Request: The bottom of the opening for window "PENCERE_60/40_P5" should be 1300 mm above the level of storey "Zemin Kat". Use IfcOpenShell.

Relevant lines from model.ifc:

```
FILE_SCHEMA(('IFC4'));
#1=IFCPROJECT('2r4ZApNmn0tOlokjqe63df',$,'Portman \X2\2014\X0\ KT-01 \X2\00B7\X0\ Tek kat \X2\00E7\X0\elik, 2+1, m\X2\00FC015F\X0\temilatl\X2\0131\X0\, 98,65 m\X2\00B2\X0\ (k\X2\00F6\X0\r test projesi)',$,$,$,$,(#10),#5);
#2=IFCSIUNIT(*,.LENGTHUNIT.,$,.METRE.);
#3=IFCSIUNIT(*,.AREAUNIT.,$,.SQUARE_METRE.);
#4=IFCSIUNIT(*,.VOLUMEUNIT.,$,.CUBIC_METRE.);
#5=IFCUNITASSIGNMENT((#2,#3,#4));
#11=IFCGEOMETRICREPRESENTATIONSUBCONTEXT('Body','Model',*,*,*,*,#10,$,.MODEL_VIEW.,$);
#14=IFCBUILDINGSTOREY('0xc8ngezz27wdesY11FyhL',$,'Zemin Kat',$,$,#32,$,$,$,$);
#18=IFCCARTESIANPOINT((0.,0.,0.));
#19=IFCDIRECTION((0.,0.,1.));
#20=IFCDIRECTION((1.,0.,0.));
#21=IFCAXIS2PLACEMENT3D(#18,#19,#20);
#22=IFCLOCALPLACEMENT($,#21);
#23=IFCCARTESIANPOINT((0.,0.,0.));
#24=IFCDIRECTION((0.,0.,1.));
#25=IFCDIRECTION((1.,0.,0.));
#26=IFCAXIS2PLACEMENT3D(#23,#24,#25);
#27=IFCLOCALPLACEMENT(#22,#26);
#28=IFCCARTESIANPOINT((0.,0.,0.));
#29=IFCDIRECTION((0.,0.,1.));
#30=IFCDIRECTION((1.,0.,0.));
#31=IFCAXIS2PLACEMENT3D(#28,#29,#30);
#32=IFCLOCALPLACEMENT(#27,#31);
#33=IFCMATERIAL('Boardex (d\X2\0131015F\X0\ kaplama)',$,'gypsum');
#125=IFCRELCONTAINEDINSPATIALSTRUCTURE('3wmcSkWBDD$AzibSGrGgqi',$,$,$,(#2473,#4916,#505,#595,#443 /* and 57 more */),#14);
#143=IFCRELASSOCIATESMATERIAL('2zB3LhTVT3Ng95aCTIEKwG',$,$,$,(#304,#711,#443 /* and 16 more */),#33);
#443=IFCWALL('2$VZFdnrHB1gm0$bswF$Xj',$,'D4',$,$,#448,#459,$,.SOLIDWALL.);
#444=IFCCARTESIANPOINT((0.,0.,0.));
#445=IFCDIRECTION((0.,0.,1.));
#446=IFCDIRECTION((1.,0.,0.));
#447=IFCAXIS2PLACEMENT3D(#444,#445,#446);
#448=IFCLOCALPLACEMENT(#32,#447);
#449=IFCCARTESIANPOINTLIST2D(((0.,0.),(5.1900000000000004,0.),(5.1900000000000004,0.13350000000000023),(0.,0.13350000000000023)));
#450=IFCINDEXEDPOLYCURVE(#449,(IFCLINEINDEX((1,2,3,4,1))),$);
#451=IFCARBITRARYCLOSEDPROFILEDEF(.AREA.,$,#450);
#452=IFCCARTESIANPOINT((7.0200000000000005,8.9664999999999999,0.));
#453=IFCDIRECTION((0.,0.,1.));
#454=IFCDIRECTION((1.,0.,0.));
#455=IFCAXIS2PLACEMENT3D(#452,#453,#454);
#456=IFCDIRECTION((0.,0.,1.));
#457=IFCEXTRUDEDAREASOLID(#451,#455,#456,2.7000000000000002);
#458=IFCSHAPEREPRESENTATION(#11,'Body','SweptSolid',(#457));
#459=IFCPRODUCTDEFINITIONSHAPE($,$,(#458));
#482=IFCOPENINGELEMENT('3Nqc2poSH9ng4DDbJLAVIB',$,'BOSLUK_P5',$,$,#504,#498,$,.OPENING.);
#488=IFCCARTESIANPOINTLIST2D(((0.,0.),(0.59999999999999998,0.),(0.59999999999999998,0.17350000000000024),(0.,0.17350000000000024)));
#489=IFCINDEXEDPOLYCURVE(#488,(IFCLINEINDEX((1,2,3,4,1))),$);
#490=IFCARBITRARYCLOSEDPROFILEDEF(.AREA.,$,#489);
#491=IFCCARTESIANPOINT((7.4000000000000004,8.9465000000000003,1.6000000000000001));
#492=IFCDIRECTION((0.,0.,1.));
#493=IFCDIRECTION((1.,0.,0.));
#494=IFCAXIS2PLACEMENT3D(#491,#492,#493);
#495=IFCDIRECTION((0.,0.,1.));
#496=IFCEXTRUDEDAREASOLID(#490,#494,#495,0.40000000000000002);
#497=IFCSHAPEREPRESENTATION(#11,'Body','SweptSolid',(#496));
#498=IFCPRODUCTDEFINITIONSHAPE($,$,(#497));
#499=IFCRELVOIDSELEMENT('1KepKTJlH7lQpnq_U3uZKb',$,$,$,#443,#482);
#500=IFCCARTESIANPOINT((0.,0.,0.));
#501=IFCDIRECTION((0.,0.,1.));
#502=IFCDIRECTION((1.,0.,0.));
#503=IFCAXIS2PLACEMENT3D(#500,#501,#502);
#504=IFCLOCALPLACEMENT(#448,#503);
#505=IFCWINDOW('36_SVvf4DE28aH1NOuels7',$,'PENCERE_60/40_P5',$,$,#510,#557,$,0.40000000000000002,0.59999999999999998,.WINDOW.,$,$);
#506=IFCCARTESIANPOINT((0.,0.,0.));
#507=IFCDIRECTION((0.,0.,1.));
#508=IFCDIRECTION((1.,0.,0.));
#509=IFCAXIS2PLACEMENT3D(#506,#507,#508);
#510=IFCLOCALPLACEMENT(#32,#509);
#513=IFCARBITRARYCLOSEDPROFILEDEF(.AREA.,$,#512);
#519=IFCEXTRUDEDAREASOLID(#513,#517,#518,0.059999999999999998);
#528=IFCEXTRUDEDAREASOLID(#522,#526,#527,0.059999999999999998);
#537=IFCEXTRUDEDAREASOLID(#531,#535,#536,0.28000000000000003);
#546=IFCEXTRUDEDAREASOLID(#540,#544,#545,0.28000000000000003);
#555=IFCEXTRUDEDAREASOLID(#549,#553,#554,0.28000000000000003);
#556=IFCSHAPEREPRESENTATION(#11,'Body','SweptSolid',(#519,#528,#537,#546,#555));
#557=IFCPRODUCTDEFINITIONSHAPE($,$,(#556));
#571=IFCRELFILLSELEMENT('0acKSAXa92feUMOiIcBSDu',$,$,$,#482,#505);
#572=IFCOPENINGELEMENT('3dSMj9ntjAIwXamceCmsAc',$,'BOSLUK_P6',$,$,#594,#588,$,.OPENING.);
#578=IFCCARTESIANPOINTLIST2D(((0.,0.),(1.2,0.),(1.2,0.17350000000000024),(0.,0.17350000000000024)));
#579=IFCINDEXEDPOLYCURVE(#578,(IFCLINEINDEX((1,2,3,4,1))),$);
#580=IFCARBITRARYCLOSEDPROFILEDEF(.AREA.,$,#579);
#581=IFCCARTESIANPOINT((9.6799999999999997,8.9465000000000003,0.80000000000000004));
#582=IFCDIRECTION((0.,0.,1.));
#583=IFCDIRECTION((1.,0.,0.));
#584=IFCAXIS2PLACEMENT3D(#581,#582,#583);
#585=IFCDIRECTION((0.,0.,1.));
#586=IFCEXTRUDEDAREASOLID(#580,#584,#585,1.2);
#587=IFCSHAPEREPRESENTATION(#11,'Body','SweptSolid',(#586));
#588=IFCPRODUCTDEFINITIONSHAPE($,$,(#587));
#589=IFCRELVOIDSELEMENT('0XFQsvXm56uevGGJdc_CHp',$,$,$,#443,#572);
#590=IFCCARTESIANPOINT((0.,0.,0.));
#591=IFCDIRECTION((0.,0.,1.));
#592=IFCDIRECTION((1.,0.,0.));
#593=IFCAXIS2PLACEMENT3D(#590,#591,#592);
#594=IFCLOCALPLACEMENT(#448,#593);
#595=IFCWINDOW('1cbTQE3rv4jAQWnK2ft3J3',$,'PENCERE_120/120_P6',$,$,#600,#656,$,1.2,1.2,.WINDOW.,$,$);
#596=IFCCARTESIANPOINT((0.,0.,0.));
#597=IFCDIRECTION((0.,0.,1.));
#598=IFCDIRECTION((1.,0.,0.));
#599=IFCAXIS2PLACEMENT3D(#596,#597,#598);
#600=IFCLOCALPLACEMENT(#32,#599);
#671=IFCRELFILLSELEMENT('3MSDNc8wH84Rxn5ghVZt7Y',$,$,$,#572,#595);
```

```python
import numpy as np
import ifcopenshell
import ifcopenshell.api.geometry
import ifcopenshell.geom
import ifcopenshell.util.element
import ifcopenshell.util.placement
import ifcopenshell.util.shape
import ifcopenshell.util.unit

model = ifcopenshell.open("model.ifc")
unit_scale = ifcopenshell.util.unit.calculate_unit_scale(model)

window = model.by_guid("36_SVvf4DE28aH1NOuels7")
opening = window.FillsVoids[0].RelatingOpeningElement
storey = ifcopenshell.util.element.get_container(window, ifc_class="IfcBuildingStorey")
level = ifcopenshell.util.placement.get_local_placement(storey.ObjectPlacement)[2, 3]

# The opening's origin need not be at the sill, so measure its lowest point.
shape = ifcopenshell.geom.create_shape(ifcopenshell.geom.settings(), opening)
bottom = ifcopenshell.util.shape.get_shape_bottom_elevation(shape, shape.geometry) / unit_scale
dz = level + 1.3 / unit_scale - bottom

shift = np.array([0.0, 0.0, dz])
# The window is not placed relative to its opening, so move both.
for product in (opening, window):
    matrix = ifcopenshell.util.placement.get_local_placement(product.ObjectPlacement)
    matrix[:3, 3] += shift
    ifcopenshell.api.geometry.edit_object_placement(model, product=product, matrix=matrix, is_si=False)

print(f"moved by {dz * unit_scale:+.3f} m")

model.write("model-out.ifc")
```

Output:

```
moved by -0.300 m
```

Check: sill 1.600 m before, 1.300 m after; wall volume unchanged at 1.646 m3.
